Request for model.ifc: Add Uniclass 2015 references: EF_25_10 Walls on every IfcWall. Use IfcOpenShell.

First a look at what the model holds.

```python
import ifcopenshell

model = ifcopenshell.open("model.ifc")
print(model.schema)
print("classifications:", [c.Name for c in model.by_type("IfcClassification")])
for ifc_class in ("IfcDoor", "IfcRoof", "IfcStair", "IfcWall", "IfcWindow"):
    print(ifc_class, len(model.by_type(ifc_class)))
```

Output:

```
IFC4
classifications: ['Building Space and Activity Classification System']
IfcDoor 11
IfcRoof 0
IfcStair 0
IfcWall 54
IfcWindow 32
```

```python
import ifcopenshell
import ifcopenshell.api.classification

model = ifcopenshell.open("model.ifc")

system = ifcopenshell.api.classification.add_classification(model, classification="Uniclass 2015")

codes = {
    "IfcWall": ("EF_25_10", "Walls"),
}
for ifc_class, (code, name) in codes.items():
    products = model.by_type(ifc_class)
    ifcopenshell.api.classification.add_reference(
        model, products=products, classification=system, identification=code, name=name
    )
    print(code, len(products))

model.write("model_rev.ifc")
```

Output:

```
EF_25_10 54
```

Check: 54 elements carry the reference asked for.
